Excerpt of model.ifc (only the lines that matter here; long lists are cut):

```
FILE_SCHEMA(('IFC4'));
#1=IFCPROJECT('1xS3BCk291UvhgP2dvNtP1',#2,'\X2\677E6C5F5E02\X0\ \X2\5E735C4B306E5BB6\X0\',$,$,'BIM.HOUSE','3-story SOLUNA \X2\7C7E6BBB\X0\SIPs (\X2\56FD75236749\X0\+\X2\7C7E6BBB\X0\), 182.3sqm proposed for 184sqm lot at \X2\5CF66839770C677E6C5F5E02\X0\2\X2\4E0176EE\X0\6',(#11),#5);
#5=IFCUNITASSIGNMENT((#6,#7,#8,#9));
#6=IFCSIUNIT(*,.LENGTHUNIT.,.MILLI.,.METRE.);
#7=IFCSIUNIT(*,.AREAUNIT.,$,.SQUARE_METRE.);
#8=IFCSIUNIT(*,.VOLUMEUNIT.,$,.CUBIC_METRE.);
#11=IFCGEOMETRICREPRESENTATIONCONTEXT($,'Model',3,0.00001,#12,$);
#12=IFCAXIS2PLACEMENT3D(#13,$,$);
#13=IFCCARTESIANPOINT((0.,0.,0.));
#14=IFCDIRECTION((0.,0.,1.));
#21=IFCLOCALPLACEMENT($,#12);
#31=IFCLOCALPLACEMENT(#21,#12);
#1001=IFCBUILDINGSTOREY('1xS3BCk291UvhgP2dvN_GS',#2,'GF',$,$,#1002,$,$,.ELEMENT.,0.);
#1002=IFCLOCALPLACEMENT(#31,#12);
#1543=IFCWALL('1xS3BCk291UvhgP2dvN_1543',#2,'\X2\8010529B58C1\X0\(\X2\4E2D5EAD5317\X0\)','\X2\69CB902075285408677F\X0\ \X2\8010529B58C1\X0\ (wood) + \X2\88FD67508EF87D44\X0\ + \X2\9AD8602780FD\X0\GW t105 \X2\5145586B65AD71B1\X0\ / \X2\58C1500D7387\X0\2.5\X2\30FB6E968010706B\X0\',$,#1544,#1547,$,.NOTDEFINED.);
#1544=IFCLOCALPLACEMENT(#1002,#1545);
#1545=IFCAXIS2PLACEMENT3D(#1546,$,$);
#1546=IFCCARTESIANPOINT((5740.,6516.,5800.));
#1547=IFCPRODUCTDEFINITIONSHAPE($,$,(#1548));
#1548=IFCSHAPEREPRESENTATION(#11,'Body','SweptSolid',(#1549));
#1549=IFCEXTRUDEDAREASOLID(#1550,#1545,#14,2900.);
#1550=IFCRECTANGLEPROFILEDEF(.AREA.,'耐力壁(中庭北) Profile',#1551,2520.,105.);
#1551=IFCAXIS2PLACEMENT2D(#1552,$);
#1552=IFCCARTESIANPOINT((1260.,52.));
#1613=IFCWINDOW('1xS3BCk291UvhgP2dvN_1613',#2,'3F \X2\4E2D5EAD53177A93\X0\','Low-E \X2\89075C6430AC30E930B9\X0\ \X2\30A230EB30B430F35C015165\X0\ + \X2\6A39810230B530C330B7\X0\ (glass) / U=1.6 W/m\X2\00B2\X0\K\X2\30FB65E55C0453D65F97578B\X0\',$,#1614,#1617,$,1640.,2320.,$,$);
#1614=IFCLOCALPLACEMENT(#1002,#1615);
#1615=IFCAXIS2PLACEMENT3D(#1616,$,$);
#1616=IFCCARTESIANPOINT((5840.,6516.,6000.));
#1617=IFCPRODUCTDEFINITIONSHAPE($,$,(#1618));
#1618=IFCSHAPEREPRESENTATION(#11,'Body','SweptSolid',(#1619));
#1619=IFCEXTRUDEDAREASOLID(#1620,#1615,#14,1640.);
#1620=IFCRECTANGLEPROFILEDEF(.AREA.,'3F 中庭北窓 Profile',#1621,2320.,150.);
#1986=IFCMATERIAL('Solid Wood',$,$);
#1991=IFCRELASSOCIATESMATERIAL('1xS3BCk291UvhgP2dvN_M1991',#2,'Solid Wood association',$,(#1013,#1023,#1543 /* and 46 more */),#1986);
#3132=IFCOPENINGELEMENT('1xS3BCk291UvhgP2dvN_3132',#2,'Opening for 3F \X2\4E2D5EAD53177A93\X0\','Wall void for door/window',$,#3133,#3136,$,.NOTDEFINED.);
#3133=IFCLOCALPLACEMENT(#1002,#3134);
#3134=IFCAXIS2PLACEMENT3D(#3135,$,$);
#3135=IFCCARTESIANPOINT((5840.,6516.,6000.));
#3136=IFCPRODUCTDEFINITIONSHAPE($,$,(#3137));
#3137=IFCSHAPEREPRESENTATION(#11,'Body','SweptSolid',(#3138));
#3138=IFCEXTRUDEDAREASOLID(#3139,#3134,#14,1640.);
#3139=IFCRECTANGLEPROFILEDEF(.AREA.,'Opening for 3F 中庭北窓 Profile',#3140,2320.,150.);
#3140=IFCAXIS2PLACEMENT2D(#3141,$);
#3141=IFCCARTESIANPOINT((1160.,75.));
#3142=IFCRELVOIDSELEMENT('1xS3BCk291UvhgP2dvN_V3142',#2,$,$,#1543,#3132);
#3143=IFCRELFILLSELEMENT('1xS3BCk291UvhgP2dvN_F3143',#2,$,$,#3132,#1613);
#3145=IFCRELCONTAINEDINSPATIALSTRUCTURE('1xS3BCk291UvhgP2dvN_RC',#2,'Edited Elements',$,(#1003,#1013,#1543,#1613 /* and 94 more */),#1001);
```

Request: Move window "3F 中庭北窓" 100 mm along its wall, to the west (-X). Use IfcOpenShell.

```python
import ifcopenshell
import ifcopenshell.api.geometry
import ifcopenshell.util.placement

model = ifcopenshell.open("model.ifc")

window = model.by_guid("1xS3BCk291UvhgP2dvN_1613")
opening = window.FillsVoids[0].RelatingOpeningElement
wall = opening.VoidsElements[0].RelatingBuildingElement

wall_matrix = ifcopenshell.util.placement.get_local_placement(wall.ObjectPlacement)
shift = wall_matrix[:3, 0] * -100.0
before = ifcopenshell.util.placement.get_local_placement(window.ObjectPlacement)[:3, 3].copy()

# The window is not placed relative to its opening, so move both.
for product in (opening, window):
    matrix = ifcopenshell.util.placement.get_local_placement(product.ObjectPlacement)
    matrix[:3, 3] += shift
    ifcopenshell.api.geometry.edit_object_placement(model, product=product, matrix=matrix, is_si=False)

after = ifcopenshell.util.placement.get_local_placement(window.ObjectPlacement)[:3, 3]
print("window moved by", (after - before).round(3) + 0.0)

model.write("model_rev.ifc")
```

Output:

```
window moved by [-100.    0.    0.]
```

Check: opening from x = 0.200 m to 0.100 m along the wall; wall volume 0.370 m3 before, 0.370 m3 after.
